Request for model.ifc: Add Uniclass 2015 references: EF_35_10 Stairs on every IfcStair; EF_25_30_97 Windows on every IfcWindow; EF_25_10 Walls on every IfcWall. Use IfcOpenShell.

First a look at what the model holds.

```python
import ifcopenshell

model = ifcopenshell.open("model.ifc")
print(model.schema)
print("classifications:", [c.Name for c in model.by_type("IfcClassification")])
for ifc_class in ("IfcDoor", "IfcRoof", "IfcStair", "IfcWall", "IfcWindow"):
    print(ifc_class, len(model.by_type(ifc_class)))
```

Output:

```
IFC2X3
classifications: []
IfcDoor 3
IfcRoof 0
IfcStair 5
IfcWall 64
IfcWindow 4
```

```python
import ifcopenshell
import ifcopenshell.api.classification

model = ifcopenshell.open("model.ifc")

# IFC2X3 requires Source and Edition and has no link from the project to the system.
system = model.create_entity("IfcClassification", Source="NBS", Edition="2015", Name="Uniclass 2015")

codes = {
    "IfcStair": ("EF_35_10", "Stairs"),
    "IfcWindow": ("EF_25_30_97", "Windows"),
    "IfcWall": ("EF_25_10", "Walls"),
}
for ifc_class, (code, name) in codes.items():
    products = model.by_type(ifc_class)
    ifcopenshell.api.classification.add_reference(
        model, products=products, classification=system, identification=code, name=name
    )
    print(code, len(products))

model.write("model_rev.ifc")
```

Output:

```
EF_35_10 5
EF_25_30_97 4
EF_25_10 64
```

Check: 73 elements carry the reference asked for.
